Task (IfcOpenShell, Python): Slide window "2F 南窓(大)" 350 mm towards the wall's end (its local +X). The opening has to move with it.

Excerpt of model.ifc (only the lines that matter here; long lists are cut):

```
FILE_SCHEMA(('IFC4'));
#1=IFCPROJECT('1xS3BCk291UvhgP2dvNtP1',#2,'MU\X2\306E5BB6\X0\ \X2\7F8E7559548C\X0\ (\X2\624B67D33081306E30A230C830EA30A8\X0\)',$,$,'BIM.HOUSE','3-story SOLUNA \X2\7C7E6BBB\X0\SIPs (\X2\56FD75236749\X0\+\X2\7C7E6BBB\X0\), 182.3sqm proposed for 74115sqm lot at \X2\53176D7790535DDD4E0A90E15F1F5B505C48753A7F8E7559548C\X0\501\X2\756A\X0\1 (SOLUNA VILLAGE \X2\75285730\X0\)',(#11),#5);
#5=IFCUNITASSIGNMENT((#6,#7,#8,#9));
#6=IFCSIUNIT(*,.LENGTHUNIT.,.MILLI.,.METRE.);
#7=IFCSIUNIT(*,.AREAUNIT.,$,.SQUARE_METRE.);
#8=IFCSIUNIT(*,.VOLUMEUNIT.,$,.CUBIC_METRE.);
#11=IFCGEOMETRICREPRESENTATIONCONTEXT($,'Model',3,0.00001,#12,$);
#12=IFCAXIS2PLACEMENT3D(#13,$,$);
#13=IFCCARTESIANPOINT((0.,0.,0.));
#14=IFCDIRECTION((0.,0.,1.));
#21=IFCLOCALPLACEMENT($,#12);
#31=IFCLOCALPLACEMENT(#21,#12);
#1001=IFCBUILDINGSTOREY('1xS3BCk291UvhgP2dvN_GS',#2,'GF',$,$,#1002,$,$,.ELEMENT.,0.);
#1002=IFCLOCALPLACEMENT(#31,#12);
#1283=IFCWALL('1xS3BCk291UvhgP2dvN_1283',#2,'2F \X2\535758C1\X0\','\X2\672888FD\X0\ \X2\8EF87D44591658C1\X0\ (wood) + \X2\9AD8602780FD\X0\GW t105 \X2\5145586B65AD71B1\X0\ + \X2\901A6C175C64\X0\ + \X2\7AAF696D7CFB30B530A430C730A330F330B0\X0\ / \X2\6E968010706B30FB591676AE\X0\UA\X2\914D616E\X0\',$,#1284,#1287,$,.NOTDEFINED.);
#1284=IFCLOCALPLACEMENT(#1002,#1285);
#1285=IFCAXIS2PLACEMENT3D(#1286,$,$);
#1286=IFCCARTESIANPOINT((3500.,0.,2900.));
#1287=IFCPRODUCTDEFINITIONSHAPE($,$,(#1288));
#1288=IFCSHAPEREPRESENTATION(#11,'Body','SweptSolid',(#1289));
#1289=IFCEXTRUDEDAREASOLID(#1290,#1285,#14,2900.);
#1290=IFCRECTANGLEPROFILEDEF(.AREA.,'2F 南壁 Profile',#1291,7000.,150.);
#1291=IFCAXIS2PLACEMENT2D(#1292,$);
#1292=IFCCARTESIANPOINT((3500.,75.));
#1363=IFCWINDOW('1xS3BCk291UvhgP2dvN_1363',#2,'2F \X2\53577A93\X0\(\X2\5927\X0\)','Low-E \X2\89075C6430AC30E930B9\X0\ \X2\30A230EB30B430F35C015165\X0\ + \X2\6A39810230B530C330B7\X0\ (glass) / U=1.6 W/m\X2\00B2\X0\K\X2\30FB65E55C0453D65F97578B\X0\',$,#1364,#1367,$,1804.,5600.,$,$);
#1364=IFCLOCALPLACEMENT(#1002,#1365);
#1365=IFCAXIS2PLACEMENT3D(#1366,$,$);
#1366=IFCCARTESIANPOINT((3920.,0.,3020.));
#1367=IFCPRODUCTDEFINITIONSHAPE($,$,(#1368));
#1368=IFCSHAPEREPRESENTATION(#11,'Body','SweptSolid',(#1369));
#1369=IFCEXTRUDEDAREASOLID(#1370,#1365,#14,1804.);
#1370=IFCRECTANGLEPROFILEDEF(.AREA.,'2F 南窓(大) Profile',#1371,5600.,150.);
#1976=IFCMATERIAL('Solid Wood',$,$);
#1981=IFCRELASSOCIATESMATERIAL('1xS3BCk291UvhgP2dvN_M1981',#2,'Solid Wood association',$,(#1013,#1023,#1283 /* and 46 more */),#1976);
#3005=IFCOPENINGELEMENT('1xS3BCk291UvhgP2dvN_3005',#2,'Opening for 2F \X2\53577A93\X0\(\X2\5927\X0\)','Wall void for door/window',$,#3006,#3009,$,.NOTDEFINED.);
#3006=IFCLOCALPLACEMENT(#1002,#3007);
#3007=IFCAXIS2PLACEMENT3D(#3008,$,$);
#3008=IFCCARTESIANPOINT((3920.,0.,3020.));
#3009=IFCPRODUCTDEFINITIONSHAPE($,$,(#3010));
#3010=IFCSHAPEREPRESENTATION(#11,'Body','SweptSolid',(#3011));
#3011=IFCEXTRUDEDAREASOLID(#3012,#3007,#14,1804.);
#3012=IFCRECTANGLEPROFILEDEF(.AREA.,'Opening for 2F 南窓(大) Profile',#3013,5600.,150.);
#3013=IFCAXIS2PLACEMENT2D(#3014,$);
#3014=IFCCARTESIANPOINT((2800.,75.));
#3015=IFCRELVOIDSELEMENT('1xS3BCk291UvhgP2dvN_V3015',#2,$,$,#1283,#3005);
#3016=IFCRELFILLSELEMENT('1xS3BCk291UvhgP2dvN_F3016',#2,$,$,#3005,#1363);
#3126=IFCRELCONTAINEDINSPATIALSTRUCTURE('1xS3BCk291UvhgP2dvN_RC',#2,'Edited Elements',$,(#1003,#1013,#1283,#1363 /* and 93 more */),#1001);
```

```python
import ifcopenshell
import ifcopenshell.api.geometry
import ifcopenshell.util.placement

model = ifcopenshell.open("model.ifc")

window = model.by_id(1363)
opening = window.FillsVoids[0].RelatingOpeningElement
wall = opening.VoidsElements[0].RelatingBuildingElement

wall_matrix = ifcopenshell.util.placement.get_local_placement(wall.ObjectPlacement)
shift = wall_matrix[:3, 0] * 350.0
before = ifcopenshell.util.placement.get_local_placement(window.ObjectPlacement)[:3, 3].copy()

# The window is not placed relative to its opening, so move both.
for product in (opening, window):
    matrix = ifcopenshell.util.placement.get_local_placement(product.ObjectPlacement)
    matrix[:3, 3] += shift
    ifcopenshell.api.geometry.edit_object_placement(model, product=product, matrix=matrix, is_si=False)

after = ifcopenshell.util.placement.get_local_placement(window.ObjectPlacement)[:3, 3]
print("window moved by", (after - before).round(3) + 0.0)

model.write("model_updated.ifc")
```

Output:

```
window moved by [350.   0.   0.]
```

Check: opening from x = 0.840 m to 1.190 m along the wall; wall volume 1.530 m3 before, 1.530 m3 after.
